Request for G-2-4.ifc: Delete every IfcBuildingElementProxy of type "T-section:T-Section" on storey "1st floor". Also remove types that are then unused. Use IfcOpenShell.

First a look at what the model holds.

```python
import ifcopenshell
import ifcopenshell.util.element

model = ifcopenshell.open("G-2-4.ifc")
print(model.schema)
storey = next(s for s in model.by_type("IfcBuildingStorey") if s.Name == "1st floor")
proxies = [e for e in ifcopenshell.util.element.get_decomposition(storey) if e.is_a("IfcBuildingElementProxy")]
seen = {}
for e in proxies:
    element_type = ifcopenshell.util.element.get_type(e)
    name = element_type.Name if element_type not in (None, e) else None
    seen[name] = seen.get(name, 0) + 1
for name, count in sorted(seen.items(), key=str):
    print(count, "x", name)
```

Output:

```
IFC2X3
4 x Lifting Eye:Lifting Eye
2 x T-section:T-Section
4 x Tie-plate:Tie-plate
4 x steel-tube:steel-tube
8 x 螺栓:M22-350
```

```python
import ifcopenshell
import ifcopenshell.api.root
import ifcopenshell.util.element

model = ifcopenshell.open("G-2-4.ifc")

storey = next(s for s in model.by_type("IfcBuildingStorey") if s.Name == "1st floor")
proxies = [e for e in ifcopenshell.util.element.get_decomposition(storey) if e.is_a("IfcBuildingElementProxy")]
targets = [e for e in proxies if (t := ifcopenshell.util.element.get_type(e)) not in (None, e) and t.Name == "T-section:T-Section"]
types = {ifcopenshell.util.element.get_type(e) for e in targets} - {None, *targets}

for e in targets:
    ifcopenshell.api.root.remove_product(model, product=e)
print(len(targets), "removed")

unused = [t for t in types if not ifcopenshell.util.element.get_types(t)]
for t in unused:
    ifcopenshell.api.root.remove_product(model, product=t)
print(len(unused), "unused types removed")

model.write("G-2-4_v2.ifc")
```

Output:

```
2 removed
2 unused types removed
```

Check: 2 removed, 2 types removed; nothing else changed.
